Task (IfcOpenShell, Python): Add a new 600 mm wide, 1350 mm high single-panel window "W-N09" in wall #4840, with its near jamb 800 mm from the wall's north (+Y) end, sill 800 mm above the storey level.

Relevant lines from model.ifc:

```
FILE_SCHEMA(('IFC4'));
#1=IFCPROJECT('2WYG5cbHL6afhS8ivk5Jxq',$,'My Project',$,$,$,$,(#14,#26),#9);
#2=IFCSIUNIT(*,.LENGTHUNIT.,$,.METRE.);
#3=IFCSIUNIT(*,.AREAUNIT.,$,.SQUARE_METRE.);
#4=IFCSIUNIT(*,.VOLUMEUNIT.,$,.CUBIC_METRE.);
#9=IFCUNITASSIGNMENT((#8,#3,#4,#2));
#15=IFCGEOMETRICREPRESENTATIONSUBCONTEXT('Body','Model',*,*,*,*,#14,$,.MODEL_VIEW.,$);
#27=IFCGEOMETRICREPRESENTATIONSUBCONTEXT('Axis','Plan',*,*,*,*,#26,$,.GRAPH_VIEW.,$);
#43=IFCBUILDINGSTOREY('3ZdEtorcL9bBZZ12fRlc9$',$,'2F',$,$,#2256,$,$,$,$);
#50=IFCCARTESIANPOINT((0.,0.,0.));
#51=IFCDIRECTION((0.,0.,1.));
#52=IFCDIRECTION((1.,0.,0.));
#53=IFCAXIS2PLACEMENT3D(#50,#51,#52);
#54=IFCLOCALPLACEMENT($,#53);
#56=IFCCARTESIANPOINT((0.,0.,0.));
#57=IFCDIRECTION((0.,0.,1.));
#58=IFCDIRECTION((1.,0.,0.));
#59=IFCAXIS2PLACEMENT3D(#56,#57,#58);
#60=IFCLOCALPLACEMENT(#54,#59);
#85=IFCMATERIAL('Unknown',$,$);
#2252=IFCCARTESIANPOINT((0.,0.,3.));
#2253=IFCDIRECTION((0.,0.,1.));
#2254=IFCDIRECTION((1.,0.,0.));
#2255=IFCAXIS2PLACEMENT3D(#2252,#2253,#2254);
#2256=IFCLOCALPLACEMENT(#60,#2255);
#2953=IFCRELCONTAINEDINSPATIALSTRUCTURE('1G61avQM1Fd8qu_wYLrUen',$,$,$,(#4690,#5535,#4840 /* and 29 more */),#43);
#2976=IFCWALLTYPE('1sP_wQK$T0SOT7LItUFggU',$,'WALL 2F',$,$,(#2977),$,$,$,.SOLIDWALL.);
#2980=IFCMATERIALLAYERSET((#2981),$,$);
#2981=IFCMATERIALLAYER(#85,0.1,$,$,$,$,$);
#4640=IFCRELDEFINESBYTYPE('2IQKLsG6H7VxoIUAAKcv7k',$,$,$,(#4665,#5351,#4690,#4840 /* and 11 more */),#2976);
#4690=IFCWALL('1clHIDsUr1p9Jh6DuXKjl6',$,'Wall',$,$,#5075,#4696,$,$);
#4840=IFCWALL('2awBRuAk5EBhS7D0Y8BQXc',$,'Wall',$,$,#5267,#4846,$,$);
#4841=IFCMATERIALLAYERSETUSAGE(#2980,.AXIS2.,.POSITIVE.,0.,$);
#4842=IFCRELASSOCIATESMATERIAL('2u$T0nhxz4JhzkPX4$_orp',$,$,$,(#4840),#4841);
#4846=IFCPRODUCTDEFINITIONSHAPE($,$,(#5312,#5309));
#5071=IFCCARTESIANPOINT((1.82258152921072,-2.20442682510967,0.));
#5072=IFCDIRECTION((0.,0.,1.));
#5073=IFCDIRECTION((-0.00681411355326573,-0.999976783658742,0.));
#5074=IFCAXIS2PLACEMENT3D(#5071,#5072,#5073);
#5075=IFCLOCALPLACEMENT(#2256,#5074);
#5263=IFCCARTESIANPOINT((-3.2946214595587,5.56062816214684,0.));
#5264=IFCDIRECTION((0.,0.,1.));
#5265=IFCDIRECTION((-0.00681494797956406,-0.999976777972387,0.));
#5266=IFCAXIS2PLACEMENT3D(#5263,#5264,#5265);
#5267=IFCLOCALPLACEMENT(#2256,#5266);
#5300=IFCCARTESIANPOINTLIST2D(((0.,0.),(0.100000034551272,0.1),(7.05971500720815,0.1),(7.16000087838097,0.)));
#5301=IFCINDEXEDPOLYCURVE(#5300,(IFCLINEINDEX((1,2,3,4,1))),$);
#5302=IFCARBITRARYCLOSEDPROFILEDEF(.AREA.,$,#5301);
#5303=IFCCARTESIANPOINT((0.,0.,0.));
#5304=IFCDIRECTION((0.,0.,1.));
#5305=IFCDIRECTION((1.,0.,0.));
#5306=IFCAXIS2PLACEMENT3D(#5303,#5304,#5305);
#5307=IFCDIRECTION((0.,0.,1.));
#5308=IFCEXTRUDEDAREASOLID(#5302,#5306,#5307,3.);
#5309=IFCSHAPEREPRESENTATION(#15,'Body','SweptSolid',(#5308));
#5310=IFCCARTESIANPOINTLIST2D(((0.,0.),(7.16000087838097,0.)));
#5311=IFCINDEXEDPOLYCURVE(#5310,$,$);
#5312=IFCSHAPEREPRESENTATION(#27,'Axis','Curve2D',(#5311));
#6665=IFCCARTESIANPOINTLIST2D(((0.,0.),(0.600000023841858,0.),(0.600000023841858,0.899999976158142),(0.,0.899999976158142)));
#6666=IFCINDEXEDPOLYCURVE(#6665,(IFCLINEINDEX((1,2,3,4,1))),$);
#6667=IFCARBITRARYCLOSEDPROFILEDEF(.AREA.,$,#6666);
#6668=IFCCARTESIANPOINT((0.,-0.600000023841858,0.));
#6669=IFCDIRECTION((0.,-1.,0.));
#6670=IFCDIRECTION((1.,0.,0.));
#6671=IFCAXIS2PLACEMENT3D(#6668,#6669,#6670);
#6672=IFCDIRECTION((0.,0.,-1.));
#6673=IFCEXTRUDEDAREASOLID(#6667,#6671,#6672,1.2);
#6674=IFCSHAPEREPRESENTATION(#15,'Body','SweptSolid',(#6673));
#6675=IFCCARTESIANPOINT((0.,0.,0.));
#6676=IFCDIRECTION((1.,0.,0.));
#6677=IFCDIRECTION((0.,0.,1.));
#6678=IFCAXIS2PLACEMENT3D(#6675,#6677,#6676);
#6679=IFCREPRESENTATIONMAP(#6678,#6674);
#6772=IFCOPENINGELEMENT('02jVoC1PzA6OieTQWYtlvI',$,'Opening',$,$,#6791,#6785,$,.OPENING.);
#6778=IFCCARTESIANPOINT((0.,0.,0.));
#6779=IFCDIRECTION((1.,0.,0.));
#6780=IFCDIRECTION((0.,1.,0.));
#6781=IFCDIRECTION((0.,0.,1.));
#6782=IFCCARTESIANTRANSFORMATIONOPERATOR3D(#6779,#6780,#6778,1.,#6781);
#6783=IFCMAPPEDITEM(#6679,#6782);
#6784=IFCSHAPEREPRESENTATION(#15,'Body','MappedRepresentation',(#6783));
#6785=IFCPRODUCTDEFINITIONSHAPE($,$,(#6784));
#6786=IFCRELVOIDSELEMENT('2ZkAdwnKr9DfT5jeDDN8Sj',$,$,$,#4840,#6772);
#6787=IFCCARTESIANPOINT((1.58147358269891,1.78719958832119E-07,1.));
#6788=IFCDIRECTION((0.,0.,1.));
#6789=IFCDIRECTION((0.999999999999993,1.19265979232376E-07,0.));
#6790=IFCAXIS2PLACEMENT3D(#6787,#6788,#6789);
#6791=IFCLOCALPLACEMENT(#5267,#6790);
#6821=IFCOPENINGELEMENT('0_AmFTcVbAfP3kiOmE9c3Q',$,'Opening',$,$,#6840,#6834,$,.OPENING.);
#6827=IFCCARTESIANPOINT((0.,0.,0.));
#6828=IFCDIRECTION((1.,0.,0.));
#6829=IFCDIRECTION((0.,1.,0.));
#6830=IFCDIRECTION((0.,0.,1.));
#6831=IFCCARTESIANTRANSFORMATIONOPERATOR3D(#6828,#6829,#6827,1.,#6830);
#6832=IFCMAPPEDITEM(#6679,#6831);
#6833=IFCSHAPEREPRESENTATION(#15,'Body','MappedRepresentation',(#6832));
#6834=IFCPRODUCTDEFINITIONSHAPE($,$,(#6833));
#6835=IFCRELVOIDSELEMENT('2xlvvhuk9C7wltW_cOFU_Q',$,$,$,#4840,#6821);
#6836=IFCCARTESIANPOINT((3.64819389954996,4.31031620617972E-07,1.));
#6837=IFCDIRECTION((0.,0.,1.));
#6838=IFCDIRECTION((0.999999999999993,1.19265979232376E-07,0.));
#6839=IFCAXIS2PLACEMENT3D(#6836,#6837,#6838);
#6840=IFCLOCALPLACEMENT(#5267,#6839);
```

```python
import numpy as np
import ifcopenshell
import ifcopenshell.api.feature
import ifcopenshell.api.geometry
import ifcopenshell.api.root
import ifcopenshell.api.spatial
import ifcopenshell.geom
import ifcopenshell.util.element
import ifcopenshell.util.placement
import ifcopenshell.util.representation
import ifcopenshell.util.shape
import ifcopenshell.util.unit

model = ifcopenshell.open("model.ifc")
unit_scale = ifcopenshell.util.unit.calculate_unit_scale(model)
settings = ifcopenshell.geom.settings()


def volume(element):
    """Net volume in cubic metres, openings subtracted."""
    shape = ifcopenshell.geom.create_shape(settings, element)
    return ifcopenshell.util.shape.get_volume(shape.geometry)


wall = model.by_guid("2awBRuAk5EBhS7D0Y8BQXc")
storey = ifcopenshell.util.element.get_container(wall, ifc_class="IfcBuildingStorey")
context = ifcopenshell.util.representation.get_context(model, "Model", "Body", "MODEL_VIEW")
before = volume(wall)

width, height, from_end, sill = 0.6, 1.35, 0.8, 0.8  # metres

# The wall runs along its own X axis, and the end named is its -X end.
wall_shape = ifcopenshell.geom.create_shape(settings, wall)
x, y, z = ifcopenshell.util.shape.get_vertices(wall_shape.geometry).T
start = x.min() + from_end
face, thickness = float(y.min()), float(y.max() - y.min())
wall_matrix = ifcopenshell.util.placement.get_local_placement(wall.ObjectPlacement)
level = ifcopenshell.util.placement.get_local_placement(storey.ObjectPlacement)[2, 3]


def in_wall(x, y):
    """Placement at x, y metres in the wall's axes, at sill height."""
    matrix = wall_matrix.copy()
    matrix[:, 3] = wall_matrix @ np.array([x / unit_scale, y / unit_scale, 0.0, 1.0])
    matrix[2, 3] = level + sill / unit_scale
    return matrix


# Opening: a box that overshoots both wall faces by 50 mm.
opening = ifcopenshell.api.root.create_entity(model, ifc_class="IfcOpeningElement", predefined_type="OPENING")
box = ifcopenshell.api.geometry.add_wall_representation(
    model, context=context, length=width, height=height, thickness=thickness + 0.1
)
ifcopenshell.api.geometry.assign_representation(model, product=opening, representation=box)
ifcopenshell.api.geometry.edit_object_placement(model, product=opening, matrix=in_wall(start, face - 0.05), is_si=False)
ifcopenshell.api.feature.add_feature(model, feature=opening, element=wall)

window = ifcopenshell.api.root.create_entity(model, ifc_class="IfcWindow", name="W-N09", predefined_type="WINDOW")
window.OverallWidth, window.OverallHeight = width / unit_scale, height / unit_scale
window.PartitioningType = "SINGLE_PANEL"
body = ifcopenshell.api.geometry.add_window_representation(
    model,
    context=context,
    overall_width=window.OverallWidth,
    overall_height=window.OverallHeight,
    partition_type="SINGLE_PANEL",
)
ifcopenshell.api.geometry.assign_representation(model, product=window, representation=body)
ifcopenshell.api.spatial.assign_container(model, products=[window], relating_structure=storey)
ifcopenshell.api.feature.add_filling(model, opening=opening, element=window)

# Centre the window in the wall's thickness.
ifcopenshell.api.geometry.edit_object_placement(model, product=window, matrix=in_wall(start, face), is_si=False)
window_shape = ifcopenshell.geom.create_shape(settings, window)
depth = ifcopenshell.util.shape.get_vertices(window_shape.geometry)[:, 1]
offset = face + thickness / 2 - (depth.min() + depth.max()) / 2
ifcopenshell.api.geometry.edit_object_placement(model, product=window, matrix=in_wall(start, offset), is_si=False)

after = volume(wall)

print(f"wall volume {before:.3f} -> {after:.3f} m3")

model.write("model_edited.ifc")
```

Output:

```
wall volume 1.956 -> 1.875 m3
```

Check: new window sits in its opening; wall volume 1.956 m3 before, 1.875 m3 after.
